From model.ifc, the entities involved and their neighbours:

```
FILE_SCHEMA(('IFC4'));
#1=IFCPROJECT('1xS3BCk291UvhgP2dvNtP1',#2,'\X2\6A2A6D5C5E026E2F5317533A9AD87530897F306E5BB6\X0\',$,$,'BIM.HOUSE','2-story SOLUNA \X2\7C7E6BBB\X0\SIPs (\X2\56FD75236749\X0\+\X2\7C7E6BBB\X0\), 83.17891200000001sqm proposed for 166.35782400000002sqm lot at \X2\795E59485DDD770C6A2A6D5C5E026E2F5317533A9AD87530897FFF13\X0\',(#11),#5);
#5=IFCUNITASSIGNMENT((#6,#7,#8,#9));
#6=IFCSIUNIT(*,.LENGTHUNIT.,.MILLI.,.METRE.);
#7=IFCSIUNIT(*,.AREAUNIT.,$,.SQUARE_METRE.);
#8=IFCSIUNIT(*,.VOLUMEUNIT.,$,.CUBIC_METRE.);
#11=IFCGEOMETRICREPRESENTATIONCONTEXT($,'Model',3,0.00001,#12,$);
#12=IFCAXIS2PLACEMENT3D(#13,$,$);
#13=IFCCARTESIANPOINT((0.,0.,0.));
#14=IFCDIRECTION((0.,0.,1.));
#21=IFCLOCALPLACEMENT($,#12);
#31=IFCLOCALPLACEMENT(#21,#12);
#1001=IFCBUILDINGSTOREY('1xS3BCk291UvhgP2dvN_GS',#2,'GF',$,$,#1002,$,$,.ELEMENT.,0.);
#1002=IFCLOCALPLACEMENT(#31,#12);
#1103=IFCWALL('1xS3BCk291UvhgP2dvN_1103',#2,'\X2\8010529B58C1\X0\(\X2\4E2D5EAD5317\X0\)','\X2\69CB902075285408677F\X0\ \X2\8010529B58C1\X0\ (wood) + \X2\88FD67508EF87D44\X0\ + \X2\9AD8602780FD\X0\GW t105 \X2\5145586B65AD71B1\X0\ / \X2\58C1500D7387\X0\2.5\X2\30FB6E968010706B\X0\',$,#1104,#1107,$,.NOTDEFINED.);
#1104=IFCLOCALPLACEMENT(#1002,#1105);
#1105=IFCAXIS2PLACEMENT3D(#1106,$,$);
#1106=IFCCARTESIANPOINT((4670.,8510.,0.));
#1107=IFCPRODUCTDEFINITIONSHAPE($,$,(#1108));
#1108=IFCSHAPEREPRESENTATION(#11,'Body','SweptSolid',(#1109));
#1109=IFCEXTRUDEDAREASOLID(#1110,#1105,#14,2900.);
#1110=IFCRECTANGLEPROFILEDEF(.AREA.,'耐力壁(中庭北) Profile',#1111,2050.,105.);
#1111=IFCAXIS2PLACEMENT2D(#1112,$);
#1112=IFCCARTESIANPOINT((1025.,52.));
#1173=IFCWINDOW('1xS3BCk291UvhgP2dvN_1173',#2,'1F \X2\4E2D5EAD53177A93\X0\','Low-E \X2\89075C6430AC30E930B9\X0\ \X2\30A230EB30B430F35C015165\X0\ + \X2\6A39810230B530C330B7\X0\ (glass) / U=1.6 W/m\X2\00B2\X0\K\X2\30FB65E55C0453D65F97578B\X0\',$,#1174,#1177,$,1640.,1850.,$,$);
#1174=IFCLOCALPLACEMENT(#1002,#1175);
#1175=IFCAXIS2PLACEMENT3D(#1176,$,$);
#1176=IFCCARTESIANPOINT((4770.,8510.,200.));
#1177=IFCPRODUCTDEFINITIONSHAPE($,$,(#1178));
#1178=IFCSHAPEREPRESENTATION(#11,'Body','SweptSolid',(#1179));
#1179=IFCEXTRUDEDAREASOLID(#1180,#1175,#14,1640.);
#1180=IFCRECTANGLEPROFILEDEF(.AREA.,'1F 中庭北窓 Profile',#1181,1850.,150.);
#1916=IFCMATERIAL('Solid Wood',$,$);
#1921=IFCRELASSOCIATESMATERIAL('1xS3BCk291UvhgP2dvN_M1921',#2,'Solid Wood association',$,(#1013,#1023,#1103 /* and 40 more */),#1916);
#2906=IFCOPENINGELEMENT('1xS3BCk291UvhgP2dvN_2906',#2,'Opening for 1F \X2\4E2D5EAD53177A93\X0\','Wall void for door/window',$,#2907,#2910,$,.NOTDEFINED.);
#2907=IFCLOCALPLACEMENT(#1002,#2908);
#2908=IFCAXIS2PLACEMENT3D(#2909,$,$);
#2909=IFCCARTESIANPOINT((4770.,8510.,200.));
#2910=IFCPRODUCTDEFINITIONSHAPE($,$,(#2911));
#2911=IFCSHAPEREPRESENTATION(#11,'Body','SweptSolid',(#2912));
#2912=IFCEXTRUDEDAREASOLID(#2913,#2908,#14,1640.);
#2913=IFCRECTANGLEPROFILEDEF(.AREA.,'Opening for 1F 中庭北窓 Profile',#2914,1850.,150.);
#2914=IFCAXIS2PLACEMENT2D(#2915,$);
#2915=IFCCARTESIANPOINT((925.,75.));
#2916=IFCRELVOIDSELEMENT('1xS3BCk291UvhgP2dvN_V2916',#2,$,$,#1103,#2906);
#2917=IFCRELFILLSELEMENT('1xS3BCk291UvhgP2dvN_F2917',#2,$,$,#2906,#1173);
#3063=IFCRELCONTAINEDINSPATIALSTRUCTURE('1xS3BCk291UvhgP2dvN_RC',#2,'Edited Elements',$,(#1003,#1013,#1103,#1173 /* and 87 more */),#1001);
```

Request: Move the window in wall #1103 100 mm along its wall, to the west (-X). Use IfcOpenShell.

```python
import ifcopenshell
import ifcopenshell.api.geometry
import ifcopenshell.util.placement

model = ifcopenshell.open("model.ifc")

window = model.by_guid("1xS3BCk291UvhgP2dvN_1173")
opening = window.FillsVoids[0].RelatingOpeningElement
wall = opening.VoidsElements[0].RelatingBuildingElement

wall_matrix = ifcopenshell.util.placement.get_local_placement(wall.ObjectPlacement)
shift = wall_matrix[:3, 0] * -100.0
before = ifcopenshell.util.placement.get_local_placement(window.ObjectPlacement)[:3, 3].copy()

# The window is not placed relative to its opening, so move both.
for product in (opening, window):
    matrix = ifcopenshell.util.placement.get_local_placement(product.ObjectPlacement)
    matrix[:3, 3] += shift
    ifcopenshell.api.geometry.edit_object_placement(model, product=product, matrix=matrix, is_si=False)

after = ifcopenshell.util.placement.get_local_placement(window.ObjectPlacement)[:3, 3]
print("window moved by", (after - before).round(3) + 0.0)

model.write("model_v2.ifc")
```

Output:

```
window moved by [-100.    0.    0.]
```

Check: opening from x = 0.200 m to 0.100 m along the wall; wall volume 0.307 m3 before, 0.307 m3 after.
